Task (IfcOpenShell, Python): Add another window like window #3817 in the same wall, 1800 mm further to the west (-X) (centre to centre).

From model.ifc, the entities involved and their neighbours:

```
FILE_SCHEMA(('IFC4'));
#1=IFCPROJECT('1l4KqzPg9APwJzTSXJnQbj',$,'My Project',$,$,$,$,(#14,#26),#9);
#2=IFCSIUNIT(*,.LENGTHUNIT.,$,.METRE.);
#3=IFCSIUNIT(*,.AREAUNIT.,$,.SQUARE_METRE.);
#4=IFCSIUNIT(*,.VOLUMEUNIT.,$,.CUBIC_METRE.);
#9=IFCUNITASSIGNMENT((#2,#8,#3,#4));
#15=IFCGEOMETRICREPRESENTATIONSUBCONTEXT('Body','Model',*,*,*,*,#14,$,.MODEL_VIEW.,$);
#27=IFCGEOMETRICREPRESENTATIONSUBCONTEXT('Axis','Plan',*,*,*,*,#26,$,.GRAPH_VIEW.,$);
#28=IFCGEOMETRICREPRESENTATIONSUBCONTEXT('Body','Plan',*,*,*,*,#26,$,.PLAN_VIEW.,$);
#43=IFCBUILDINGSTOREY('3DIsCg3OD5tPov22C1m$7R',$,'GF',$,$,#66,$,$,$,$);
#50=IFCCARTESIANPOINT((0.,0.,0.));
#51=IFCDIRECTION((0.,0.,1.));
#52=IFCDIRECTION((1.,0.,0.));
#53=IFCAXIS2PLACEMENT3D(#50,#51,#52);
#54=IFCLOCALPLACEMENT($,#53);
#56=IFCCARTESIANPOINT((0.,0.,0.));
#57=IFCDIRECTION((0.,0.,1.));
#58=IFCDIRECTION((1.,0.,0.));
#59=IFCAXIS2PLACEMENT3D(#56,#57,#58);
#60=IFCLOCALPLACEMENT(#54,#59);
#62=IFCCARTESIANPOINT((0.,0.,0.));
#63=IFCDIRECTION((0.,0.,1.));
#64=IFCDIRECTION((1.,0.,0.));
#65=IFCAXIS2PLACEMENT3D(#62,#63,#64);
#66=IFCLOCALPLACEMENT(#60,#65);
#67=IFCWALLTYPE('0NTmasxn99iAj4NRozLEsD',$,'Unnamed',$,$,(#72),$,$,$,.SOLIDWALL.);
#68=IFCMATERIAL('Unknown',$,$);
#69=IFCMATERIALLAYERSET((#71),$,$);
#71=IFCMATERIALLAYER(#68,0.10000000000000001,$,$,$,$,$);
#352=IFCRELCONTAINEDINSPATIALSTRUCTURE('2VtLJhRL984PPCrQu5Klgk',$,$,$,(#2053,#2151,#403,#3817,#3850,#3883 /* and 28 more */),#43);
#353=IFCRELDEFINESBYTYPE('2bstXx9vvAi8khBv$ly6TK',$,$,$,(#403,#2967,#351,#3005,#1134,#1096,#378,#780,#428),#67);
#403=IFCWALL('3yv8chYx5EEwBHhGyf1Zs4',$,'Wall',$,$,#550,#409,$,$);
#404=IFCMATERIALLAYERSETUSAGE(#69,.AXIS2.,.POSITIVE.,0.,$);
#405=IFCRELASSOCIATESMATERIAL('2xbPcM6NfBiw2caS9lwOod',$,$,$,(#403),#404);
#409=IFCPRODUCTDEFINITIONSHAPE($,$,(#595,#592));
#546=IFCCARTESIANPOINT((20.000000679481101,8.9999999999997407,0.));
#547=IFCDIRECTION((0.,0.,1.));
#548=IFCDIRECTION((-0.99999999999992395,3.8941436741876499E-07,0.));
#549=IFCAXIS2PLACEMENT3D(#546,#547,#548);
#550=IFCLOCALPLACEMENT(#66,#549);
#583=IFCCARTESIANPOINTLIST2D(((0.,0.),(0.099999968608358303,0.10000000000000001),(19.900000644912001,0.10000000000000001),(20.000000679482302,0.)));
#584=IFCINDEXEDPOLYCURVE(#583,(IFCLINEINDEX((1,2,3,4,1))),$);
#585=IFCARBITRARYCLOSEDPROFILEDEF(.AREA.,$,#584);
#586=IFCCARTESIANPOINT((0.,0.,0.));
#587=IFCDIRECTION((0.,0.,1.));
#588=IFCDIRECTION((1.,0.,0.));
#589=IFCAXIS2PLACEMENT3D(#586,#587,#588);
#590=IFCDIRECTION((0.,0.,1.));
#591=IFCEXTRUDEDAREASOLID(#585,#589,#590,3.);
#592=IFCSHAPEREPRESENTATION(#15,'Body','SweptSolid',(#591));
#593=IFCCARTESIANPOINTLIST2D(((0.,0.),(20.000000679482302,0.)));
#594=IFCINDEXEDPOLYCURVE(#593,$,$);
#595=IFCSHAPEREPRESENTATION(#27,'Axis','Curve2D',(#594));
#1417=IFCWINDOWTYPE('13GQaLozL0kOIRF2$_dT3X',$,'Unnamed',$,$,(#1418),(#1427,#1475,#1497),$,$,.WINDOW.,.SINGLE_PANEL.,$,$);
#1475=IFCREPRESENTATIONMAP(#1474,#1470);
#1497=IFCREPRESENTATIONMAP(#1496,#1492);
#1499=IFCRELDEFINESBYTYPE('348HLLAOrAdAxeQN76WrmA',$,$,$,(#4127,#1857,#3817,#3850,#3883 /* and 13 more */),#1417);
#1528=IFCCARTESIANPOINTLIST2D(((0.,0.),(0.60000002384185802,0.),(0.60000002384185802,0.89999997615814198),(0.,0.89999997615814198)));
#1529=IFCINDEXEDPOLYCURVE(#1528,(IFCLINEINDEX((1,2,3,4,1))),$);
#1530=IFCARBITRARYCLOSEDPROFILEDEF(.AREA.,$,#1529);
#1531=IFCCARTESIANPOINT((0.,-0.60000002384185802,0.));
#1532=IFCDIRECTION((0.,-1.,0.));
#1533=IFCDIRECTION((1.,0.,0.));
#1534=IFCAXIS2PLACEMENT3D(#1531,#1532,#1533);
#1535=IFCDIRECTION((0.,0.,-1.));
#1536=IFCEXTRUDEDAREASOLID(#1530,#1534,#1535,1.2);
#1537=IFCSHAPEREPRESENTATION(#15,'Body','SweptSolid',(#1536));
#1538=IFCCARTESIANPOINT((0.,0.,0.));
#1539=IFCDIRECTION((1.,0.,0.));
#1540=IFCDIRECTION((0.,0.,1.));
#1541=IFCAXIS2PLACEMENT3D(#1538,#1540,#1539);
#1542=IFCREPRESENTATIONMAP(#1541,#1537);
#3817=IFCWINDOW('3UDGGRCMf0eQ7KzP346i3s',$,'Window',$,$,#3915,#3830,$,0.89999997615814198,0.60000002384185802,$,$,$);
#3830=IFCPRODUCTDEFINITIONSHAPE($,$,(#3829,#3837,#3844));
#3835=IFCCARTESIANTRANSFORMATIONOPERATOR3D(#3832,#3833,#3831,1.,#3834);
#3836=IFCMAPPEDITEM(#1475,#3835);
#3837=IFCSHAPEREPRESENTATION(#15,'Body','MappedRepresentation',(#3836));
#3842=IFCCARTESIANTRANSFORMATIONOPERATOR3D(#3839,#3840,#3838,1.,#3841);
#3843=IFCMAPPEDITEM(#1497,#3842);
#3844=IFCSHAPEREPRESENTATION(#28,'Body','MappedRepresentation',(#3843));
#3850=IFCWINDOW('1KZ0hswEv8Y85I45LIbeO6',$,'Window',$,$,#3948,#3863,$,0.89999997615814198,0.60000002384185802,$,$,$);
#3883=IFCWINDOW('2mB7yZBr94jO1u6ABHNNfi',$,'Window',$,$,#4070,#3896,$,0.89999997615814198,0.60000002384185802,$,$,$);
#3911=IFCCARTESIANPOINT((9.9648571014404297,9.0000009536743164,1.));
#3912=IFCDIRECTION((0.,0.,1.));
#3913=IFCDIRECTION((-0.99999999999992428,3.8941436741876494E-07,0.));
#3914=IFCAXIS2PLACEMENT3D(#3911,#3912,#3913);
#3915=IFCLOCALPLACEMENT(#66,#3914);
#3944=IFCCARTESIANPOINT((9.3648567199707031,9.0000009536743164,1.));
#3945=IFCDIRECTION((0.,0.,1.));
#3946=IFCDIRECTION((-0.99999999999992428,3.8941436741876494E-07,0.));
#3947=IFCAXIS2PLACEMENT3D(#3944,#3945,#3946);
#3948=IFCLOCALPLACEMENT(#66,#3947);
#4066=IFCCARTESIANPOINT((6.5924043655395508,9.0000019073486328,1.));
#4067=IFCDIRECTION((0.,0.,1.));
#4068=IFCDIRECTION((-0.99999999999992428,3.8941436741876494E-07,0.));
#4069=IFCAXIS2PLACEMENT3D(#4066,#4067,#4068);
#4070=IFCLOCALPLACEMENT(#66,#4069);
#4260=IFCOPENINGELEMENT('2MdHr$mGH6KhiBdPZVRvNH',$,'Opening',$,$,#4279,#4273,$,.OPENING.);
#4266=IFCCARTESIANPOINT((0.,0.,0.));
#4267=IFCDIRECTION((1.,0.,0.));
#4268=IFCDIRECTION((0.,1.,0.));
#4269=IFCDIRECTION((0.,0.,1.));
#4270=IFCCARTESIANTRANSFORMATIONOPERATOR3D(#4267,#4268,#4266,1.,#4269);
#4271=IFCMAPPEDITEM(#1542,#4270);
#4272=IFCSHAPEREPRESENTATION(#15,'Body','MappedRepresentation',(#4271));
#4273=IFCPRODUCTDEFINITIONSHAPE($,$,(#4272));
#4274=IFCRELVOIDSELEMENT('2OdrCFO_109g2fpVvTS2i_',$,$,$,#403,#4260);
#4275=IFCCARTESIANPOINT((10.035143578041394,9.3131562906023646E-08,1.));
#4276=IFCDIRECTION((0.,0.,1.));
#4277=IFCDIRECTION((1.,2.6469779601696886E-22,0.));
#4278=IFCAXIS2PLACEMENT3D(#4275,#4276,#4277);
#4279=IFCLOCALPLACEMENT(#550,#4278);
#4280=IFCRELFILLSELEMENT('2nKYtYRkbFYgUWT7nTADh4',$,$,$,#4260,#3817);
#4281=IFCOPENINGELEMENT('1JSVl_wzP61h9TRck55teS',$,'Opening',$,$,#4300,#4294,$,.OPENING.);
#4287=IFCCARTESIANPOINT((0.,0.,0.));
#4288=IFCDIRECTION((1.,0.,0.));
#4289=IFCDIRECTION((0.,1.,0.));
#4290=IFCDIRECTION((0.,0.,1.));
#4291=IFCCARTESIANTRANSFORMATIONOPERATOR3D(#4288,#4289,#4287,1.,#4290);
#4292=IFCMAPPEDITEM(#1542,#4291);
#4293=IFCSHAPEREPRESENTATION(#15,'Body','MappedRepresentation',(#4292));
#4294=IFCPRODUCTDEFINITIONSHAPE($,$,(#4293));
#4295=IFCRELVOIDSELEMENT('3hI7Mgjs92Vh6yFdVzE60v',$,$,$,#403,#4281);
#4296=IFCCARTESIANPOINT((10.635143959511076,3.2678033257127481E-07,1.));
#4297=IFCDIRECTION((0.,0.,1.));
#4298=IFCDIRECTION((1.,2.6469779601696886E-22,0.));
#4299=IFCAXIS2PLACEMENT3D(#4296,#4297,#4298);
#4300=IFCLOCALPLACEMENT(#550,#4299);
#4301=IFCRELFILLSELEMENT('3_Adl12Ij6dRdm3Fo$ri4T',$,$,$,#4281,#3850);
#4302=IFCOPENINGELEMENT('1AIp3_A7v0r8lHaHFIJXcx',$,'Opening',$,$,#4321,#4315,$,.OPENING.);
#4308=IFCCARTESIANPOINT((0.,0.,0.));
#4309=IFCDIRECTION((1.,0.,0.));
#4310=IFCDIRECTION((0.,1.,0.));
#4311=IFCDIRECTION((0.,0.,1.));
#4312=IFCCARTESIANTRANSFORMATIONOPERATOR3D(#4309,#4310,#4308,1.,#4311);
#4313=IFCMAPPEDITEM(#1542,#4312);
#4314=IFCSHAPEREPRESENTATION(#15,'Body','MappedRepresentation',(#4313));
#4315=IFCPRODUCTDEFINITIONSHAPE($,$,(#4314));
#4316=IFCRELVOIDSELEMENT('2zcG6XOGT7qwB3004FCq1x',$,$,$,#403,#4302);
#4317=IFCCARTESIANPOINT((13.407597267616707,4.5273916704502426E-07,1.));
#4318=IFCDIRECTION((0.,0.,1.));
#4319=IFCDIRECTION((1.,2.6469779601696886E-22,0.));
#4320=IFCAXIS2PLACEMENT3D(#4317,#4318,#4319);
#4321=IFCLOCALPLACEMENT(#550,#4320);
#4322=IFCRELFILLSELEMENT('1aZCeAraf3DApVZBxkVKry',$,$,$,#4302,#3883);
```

```python
import ifcopenshell
import ifcopenshell.api.feature
import ifcopenshell.api.geometry
import ifcopenshell.api.root
import ifcopenshell.geom
import ifcopenshell.util.element
import ifcopenshell.util.placement
import ifcopenshell.util.shape

model = ifcopenshell.open("model.ifc")
settings = ifcopenshell.geom.settings()


def volume(element):
    """Net volume in cubic metres, openings subtracted."""
    shape = ifcopenshell.geom.create_shape(settings, element)
    return ifcopenshell.util.shape.get_volume(shape.geometry)


window = model.by_id(3817)
opening = window.FillsVoids[0].RelatingOpeningElement
wall = opening.VoidsElements[0].RelatingBuildingElement
before = volume(wall)
shift = ifcopenshell.util.placement.get_local_placement(wall.ObjectPlacement)[:3, 0] * 1.8

# copy_class copies the void relationship, type, container and properties, but no geometry.
new_opening = ifcopenshell.api.root.copy_class(model, product=opening)
new_opening.Representation = ifcopenshell.util.element.copy_deep(
    model, opening.Representation, exclude=["IfcGeometricRepresentationContext", "IfcRepresentationMap"]
)
new_window = ifcopenshell.api.root.copy_class(model, product=window)
new_window.Representation = ifcopenshell.util.element.copy_deep(
    model, window.Representation, exclude=["IfcGeometricRepresentationContext", "IfcRepresentationMap"]
)
ifcopenshell.api.feature.add_filling(model, opening=new_opening, element=new_window)

for old, new in ((opening, new_opening), (window, new_window)):
    matrix = ifcopenshell.util.placement.get_local_placement(old.ObjectPlacement)
    matrix[:3, 3] += shift
    ifcopenshell.api.geometry.edit_object_placement(model, product=new, matrix=matrix, is_si=False)

after = volume(wall)

print(f"wall volume {before:.3f} -> {after:.3f} m3")

model.write("model_updated.ifc")
```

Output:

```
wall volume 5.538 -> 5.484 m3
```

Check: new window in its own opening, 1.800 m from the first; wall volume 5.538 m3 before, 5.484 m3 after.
